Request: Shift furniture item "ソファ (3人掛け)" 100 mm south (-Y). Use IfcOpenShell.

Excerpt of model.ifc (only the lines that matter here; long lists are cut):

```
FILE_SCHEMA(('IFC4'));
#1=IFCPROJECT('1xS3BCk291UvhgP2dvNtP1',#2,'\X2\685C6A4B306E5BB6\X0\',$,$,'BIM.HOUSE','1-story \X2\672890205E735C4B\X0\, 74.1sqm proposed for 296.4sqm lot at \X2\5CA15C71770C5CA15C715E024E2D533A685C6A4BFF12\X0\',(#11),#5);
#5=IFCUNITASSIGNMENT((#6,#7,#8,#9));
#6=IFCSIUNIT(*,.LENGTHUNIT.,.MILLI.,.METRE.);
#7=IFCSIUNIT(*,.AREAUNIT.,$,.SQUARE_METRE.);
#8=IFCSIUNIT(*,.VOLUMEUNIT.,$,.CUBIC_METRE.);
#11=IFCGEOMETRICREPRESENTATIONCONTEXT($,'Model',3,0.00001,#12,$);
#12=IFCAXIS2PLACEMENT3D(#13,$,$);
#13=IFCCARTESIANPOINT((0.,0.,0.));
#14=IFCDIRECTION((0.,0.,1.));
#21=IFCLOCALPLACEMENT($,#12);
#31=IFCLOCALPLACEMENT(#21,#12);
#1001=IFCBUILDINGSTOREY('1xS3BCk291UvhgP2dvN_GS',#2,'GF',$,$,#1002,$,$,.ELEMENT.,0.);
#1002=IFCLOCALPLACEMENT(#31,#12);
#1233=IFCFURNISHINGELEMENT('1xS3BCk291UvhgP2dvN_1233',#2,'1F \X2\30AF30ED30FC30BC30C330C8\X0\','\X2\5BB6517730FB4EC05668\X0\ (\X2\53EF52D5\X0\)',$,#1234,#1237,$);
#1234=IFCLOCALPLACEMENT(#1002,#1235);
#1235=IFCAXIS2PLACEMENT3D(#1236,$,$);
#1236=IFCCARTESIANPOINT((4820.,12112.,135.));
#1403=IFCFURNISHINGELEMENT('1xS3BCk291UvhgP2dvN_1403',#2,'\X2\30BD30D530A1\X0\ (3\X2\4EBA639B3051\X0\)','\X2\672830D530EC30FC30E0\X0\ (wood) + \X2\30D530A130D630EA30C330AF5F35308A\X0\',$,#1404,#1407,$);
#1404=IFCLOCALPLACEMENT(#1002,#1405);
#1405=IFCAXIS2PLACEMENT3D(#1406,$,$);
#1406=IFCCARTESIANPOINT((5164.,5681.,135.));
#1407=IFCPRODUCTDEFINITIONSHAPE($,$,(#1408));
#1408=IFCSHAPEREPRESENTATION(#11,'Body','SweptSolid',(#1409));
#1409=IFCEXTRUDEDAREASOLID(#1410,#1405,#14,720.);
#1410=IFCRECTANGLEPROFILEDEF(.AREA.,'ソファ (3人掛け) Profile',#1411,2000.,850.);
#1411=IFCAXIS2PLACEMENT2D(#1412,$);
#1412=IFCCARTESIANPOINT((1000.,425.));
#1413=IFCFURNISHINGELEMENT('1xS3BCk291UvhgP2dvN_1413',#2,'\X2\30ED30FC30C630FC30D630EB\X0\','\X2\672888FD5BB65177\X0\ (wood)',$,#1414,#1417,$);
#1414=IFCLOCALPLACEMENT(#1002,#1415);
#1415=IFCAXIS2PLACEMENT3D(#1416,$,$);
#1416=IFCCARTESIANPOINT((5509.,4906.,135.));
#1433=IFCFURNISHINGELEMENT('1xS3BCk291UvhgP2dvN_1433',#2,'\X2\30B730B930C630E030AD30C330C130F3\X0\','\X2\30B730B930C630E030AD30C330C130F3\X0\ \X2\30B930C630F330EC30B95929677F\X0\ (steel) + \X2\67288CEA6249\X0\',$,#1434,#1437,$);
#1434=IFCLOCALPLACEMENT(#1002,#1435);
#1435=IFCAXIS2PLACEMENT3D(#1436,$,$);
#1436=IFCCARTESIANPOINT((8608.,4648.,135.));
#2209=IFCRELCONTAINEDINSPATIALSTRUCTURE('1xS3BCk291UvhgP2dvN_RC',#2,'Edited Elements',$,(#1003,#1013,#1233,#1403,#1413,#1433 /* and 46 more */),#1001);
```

```python
import ifcopenshell
import ifcopenshell.api.geometry
import ifcopenshell.util.placement

model = ifcopenshell.open("model.ifc")

item = model.by_id(1403)
matrix = ifcopenshell.util.placement.get_local_placement(item.ObjectPlacement)
matrix[1, 3] -= 100.0
ifcopenshell.api.geometry.edit_object_placement(model, product=item, matrix=matrix, is_si=False)

print(ifcopenshell.util.placement.get_local_placement(item.ObjectPlacement).round(3) + 0.0)

model.write("model_edited.ifc")
```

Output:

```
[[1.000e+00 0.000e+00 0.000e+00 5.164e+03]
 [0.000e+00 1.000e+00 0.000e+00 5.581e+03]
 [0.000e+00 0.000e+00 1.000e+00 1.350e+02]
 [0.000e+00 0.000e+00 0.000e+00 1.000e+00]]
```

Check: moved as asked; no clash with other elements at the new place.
